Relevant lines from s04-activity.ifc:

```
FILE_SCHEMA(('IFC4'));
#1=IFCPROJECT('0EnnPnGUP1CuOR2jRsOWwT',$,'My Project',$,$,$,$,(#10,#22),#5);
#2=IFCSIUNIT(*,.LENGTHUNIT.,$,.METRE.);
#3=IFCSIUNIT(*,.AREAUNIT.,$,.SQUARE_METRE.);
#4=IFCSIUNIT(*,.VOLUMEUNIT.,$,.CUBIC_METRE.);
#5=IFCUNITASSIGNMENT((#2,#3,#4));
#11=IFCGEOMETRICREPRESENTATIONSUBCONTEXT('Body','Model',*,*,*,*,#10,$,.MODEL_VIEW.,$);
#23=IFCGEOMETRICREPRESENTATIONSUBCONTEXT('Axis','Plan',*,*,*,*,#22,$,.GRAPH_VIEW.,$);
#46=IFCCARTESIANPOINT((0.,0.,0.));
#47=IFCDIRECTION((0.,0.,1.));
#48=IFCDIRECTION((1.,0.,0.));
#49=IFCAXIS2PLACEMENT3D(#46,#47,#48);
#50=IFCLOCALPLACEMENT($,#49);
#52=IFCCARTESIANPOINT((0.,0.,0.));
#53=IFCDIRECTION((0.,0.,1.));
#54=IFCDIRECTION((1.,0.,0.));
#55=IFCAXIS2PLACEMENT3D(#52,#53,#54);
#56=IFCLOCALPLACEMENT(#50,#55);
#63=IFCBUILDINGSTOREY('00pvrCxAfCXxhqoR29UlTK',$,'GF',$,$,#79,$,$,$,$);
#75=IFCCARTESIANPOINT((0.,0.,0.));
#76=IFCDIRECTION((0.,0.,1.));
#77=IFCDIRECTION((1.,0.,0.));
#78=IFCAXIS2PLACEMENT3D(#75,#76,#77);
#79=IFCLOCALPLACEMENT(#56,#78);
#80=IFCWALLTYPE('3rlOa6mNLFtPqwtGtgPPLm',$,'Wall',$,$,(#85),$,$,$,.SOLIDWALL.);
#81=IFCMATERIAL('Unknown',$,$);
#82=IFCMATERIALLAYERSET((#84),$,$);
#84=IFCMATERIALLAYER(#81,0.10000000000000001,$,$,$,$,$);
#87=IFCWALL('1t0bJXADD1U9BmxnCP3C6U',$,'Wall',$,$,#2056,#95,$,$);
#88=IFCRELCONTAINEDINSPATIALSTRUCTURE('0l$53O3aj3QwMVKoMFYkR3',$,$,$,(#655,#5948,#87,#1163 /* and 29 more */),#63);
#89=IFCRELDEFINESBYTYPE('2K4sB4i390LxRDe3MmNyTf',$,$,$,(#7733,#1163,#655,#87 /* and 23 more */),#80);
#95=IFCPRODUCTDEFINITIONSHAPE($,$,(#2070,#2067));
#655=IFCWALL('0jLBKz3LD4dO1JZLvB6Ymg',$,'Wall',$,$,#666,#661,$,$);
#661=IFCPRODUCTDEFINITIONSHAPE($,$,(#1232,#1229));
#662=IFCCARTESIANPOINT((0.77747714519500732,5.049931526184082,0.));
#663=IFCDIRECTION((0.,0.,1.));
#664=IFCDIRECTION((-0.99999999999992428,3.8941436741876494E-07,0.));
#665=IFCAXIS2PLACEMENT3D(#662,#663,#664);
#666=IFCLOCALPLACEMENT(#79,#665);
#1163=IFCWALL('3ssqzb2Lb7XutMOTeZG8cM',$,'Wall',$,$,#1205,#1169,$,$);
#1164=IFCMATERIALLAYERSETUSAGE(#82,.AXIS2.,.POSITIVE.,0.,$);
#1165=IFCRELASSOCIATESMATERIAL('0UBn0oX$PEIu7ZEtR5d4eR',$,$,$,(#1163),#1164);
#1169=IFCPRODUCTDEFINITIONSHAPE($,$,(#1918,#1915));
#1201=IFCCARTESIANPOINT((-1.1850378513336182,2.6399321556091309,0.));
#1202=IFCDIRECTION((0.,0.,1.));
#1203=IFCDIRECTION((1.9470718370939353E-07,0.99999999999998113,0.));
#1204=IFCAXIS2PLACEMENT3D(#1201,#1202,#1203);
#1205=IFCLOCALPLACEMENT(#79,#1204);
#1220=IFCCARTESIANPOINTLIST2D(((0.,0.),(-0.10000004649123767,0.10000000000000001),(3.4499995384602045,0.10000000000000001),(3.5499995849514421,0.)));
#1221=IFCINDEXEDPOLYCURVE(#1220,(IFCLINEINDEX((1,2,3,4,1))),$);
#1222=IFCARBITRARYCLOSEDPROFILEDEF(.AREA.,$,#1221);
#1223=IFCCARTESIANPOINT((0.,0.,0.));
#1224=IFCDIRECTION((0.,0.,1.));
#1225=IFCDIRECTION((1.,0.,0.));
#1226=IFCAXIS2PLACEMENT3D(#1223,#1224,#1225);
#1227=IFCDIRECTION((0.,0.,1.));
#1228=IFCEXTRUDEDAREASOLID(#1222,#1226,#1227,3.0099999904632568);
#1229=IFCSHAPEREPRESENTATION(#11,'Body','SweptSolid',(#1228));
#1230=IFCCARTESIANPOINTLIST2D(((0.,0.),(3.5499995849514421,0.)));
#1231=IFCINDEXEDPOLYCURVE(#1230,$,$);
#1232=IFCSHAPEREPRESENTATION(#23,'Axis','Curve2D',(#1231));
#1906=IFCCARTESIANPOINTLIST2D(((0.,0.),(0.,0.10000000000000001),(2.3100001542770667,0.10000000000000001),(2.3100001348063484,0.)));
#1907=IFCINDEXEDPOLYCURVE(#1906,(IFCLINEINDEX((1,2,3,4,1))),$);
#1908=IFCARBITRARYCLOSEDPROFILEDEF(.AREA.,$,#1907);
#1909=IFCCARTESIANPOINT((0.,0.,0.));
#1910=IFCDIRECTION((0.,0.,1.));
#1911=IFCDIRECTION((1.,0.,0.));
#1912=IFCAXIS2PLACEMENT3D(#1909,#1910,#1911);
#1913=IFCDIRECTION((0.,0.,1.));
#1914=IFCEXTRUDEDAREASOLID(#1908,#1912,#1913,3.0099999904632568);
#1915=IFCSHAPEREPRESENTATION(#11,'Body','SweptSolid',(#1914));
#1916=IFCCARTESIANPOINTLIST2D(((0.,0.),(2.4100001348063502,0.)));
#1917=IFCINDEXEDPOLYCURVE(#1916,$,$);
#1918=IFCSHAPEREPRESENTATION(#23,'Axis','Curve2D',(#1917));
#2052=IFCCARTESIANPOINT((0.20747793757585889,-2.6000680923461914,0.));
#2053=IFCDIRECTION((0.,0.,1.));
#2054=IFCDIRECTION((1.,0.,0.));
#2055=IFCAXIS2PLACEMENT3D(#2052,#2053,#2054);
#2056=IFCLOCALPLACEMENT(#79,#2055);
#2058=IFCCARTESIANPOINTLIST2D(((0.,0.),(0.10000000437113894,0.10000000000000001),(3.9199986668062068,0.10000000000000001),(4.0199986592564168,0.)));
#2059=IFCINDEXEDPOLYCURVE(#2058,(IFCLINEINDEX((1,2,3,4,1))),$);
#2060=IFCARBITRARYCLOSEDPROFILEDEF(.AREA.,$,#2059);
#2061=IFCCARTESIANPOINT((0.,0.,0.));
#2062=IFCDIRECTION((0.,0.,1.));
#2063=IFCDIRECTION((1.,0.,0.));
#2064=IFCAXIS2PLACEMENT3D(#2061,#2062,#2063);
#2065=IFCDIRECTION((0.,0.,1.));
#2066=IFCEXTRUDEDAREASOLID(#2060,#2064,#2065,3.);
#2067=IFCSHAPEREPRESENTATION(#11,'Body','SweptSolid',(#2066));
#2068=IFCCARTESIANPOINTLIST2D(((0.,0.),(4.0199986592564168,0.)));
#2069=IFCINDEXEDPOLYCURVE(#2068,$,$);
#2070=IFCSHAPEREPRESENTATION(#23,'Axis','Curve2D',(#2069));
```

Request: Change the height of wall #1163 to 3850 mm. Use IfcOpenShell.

```python
import ifcopenshell
import ifcopenshell.geom
import ifcopenshell.util.representation
import ifcopenshell.util.shape
import ifcopenshell.util.unit

model = ifcopenshell.open("s04-activity.ifc")
unit_scale = ifcopenshell.util.unit.calculate_unit_scale(model)
settings = ifcopenshell.geom.settings()


def volume(element):
    """Net volume in cubic metres, openings subtracted."""
    shape = ifcopenshell.geom.create_shape(settings, element)
    return ifcopenshell.util.shape.get_volume(shape.geometry)


wall = model.by_guid("3ssqzb2Lb7XutMOTeZG8cM")
before = volume(wall)

body = ifcopenshell.util.representation.get_representation(wall, "Model", "Body")
solid = body.Items[0]
old_height = solid.Depth
solid.Depth = 3.85 / unit_scale
after = volume(wall)

print(f"height {old_height:g} -> {solid.Depth:g}, volume {before:.3f} -> {after:.3f} m3")

model.write("s04-activity_v2.ifc")
```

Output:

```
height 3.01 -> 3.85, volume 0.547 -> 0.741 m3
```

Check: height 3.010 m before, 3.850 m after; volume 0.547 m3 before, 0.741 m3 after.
